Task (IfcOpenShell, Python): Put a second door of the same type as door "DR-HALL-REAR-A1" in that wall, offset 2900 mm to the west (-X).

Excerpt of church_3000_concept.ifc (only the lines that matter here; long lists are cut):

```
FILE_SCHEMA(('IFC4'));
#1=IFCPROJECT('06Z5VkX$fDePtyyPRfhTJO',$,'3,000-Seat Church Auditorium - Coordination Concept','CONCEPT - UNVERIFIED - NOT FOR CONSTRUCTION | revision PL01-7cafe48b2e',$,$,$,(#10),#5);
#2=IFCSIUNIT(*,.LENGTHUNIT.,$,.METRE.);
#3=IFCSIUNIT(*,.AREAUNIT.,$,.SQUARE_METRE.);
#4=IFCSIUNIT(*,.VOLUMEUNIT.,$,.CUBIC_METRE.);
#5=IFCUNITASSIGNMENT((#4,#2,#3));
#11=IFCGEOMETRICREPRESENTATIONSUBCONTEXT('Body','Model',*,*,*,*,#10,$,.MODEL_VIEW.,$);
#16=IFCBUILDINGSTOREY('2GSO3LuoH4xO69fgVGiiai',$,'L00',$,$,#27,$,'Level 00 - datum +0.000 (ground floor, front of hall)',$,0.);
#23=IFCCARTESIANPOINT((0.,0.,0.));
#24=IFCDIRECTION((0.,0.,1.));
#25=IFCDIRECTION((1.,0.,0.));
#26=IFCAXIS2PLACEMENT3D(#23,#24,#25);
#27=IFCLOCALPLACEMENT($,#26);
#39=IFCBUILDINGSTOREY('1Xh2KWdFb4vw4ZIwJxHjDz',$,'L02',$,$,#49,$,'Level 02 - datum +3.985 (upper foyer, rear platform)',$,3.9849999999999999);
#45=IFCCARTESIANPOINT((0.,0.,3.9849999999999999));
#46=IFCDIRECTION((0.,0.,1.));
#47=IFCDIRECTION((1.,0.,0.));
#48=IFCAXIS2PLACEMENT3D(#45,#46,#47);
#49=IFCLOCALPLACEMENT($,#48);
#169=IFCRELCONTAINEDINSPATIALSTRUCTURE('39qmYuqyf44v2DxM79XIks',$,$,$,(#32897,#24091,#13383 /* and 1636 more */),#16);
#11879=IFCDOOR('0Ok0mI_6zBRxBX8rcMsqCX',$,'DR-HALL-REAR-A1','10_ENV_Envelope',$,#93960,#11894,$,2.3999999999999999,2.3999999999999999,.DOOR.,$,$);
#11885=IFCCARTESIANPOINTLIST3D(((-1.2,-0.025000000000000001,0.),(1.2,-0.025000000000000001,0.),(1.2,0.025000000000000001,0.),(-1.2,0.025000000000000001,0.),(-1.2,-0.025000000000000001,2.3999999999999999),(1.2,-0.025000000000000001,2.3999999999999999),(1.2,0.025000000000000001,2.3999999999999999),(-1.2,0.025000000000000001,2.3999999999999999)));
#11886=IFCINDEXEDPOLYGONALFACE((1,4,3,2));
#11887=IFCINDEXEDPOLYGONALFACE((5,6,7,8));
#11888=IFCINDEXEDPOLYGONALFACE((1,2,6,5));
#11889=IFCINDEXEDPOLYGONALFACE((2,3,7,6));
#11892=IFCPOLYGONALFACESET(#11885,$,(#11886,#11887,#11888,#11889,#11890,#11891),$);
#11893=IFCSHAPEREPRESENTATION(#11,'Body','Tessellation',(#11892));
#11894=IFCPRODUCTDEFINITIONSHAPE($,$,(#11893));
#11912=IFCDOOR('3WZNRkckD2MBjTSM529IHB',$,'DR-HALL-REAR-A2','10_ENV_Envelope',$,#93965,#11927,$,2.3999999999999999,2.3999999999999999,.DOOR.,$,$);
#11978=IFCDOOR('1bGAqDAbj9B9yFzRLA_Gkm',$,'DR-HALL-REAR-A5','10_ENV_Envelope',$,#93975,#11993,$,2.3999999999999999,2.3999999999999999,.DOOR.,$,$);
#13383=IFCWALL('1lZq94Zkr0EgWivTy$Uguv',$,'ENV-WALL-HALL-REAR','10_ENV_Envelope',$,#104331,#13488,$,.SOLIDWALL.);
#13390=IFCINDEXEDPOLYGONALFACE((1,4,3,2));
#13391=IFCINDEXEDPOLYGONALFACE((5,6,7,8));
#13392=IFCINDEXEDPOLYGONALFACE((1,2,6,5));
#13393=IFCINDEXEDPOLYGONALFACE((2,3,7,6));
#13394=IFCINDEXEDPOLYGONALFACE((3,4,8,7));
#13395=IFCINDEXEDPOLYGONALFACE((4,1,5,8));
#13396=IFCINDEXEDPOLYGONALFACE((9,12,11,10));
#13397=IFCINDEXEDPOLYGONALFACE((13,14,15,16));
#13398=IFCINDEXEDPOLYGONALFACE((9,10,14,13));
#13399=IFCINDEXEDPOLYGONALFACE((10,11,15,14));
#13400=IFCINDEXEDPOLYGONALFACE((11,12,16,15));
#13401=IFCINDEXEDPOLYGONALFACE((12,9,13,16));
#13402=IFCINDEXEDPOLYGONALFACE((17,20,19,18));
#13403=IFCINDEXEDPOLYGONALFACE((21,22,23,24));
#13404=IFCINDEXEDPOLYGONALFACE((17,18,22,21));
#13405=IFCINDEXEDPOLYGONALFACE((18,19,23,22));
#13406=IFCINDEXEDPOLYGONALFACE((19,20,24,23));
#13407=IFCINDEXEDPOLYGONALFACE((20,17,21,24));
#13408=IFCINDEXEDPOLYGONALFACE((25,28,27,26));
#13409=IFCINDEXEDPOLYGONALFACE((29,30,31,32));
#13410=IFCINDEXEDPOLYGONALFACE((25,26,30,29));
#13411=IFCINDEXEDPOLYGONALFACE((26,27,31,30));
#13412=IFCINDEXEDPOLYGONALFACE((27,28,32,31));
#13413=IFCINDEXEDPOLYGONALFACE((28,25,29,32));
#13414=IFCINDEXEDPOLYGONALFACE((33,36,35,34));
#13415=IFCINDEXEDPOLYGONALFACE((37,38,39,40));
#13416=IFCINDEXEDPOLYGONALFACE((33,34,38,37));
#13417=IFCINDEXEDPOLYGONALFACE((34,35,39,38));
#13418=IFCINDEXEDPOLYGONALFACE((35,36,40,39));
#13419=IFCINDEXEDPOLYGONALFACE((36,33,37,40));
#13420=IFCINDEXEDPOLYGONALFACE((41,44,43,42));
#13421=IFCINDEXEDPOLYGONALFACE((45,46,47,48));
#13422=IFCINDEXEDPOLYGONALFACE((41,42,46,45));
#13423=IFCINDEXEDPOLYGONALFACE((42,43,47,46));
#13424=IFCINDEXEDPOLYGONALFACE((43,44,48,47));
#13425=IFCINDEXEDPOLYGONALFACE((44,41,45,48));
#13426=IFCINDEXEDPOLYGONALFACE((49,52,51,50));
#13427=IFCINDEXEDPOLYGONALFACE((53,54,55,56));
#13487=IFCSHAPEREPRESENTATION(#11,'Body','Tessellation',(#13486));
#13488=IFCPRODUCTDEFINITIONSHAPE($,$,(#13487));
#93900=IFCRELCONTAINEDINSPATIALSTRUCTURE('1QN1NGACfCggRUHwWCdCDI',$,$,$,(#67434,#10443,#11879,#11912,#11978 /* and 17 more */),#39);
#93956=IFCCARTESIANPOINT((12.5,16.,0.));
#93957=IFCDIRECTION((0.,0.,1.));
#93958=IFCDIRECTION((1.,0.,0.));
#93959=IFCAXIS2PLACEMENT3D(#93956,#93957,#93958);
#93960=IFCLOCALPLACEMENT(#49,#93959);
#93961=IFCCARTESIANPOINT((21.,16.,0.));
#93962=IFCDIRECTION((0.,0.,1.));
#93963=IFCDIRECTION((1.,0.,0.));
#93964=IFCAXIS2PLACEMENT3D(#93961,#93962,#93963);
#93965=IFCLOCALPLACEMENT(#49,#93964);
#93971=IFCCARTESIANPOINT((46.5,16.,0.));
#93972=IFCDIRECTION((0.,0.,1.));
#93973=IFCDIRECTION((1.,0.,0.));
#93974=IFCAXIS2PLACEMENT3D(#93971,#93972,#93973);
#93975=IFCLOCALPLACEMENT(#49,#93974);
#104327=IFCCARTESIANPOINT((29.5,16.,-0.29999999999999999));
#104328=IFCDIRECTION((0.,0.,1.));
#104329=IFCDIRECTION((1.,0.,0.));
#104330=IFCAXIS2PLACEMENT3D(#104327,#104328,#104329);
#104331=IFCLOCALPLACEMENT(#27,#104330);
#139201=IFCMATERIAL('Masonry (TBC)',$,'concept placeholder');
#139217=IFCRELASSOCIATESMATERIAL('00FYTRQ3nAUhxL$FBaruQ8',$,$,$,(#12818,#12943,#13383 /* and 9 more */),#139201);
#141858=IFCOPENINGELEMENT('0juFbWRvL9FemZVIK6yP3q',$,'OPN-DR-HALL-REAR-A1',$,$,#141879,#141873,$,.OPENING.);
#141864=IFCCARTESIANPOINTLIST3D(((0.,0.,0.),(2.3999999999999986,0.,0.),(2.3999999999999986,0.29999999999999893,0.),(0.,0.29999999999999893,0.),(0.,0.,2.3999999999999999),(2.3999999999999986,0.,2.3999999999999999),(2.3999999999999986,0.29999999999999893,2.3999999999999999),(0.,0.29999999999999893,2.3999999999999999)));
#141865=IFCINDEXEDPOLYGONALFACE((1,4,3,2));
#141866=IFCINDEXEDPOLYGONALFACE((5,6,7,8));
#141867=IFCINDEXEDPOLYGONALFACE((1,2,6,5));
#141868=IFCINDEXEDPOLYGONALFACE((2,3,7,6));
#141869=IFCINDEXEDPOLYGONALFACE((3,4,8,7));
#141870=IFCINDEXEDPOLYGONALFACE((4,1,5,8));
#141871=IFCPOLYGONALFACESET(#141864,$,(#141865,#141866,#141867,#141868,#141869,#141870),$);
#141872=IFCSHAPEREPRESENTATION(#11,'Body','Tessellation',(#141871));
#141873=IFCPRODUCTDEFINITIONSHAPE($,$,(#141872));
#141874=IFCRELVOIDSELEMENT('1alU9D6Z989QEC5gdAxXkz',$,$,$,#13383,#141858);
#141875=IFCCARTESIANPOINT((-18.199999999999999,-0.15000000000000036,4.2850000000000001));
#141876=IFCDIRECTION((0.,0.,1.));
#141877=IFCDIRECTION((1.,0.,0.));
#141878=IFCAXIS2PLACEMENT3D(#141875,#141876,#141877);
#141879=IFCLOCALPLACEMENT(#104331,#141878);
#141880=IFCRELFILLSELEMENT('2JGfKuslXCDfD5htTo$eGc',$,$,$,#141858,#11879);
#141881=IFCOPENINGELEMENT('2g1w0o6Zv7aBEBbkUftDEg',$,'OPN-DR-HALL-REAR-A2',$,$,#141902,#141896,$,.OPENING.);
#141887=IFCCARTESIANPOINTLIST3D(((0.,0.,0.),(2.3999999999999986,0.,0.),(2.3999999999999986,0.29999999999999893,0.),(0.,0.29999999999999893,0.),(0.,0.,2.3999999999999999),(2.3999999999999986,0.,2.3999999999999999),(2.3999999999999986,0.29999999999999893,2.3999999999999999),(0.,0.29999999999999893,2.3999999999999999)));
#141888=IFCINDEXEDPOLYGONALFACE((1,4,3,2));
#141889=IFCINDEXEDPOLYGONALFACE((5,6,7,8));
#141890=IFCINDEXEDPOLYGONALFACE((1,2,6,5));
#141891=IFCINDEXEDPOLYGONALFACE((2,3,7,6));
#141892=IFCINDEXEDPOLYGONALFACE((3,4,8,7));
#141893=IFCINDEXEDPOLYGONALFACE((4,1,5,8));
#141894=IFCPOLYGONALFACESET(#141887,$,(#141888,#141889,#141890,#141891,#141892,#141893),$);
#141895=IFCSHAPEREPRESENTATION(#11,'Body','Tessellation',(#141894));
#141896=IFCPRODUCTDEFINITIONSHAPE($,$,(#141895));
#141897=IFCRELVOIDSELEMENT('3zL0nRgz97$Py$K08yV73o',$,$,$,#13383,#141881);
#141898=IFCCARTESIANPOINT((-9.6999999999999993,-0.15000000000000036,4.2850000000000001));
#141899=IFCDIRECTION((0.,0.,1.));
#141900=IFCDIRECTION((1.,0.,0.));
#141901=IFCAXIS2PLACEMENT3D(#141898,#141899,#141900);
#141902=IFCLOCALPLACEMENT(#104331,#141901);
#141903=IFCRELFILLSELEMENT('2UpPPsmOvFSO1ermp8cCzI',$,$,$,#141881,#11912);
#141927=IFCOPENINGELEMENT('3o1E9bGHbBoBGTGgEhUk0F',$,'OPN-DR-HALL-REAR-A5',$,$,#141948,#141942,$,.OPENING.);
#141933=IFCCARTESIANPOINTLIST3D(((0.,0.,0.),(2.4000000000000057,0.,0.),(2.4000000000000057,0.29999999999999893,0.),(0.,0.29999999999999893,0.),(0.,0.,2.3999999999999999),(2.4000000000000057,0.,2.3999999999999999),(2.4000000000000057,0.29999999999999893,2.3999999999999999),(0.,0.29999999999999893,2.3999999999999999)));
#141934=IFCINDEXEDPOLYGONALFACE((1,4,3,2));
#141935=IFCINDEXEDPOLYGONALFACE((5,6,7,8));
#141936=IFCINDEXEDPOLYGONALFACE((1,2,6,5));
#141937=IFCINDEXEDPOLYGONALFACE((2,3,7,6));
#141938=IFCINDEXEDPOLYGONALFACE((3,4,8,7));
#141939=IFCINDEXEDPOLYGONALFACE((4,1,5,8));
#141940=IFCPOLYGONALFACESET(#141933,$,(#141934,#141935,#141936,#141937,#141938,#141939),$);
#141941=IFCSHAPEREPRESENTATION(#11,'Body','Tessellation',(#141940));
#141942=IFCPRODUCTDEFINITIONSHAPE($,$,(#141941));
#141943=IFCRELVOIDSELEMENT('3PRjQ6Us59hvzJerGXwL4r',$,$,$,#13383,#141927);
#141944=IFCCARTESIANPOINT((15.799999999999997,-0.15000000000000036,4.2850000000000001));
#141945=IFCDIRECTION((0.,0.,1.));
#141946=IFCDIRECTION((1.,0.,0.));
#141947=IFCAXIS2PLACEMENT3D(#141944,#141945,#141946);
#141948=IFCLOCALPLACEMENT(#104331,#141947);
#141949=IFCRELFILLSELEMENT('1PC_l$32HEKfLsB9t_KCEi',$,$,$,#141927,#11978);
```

```python
import ifcopenshell
import ifcopenshell.api.feature
import ifcopenshell.api.geometry
import ifcopenshell.api.root
import ifcopenshell.geom
import ifcopenshell.util.element
import ifcopenshell.util.placement
import ifcopenshell.util.shape

model = ifcopenshell.open("church_3000_concept.ifc")
settings = ifcopenshell.geom.settings()


def volume(element):
    """Net volume in cubic metres, openings subtracted."""
    shape = ifcopenshell.geom.create_shape(settings, element)
    return ifcopenshell.util.shape.get_volume(shape.geometry)


door = model.by_guid("0Ok0mI_6zBRxBX8rcMsqCX")
opening = door.FillsVoids[0].RelatingOpeningElement
wall = opening.VoidsElements[0].RelatingBuildingElement
before = volume(wall)
shift = ifcopenshell.util.placement.get_local_placement(wall.ObjectPlacement)[:3, 0] * -2.9

# copy_class copies the void relationship, type, container and properties, but no geometry.
new_opening = ifcopenshell.api.root.copy_class(model, product=opening)
new_opening.Representation = ifcopenshell.util.element.copy_deep(
    model, opening.Representation, exclude=["IfcGeometricRepresentationContext", "IfcRepresentationMap"]
)
new_door = ifcopenshell.api.root.copy_class(model, product=door)
new_door.Representation = ifcopenshell.util.element.copy_deep(
    model, door.Representation, exclude=["IfcGeometricRepresentationContext", "IfcRepresentationMap"]
)
ifcopenshell.api.feature.add_filling(model, opening=new_opening, element=new_door)

for old, new in ((opening, new_opening), (door, new_door)):
    matrix = ifcopenshell.util.placement.get_local_placement(old.ObjectPlacement)
    matrix[:3, 3] += shift
    ifcopenshell.api.geometry.edit_object_placement(model, product=new, matrix=matrix, is_si=False)

after = volume(wall)

print(f"wall volume {before:.3f} -> {after:.3f} m3")

model.write("church_3000_concept_rev.ifc")
```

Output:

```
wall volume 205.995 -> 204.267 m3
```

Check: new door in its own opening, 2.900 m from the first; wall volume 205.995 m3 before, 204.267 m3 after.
